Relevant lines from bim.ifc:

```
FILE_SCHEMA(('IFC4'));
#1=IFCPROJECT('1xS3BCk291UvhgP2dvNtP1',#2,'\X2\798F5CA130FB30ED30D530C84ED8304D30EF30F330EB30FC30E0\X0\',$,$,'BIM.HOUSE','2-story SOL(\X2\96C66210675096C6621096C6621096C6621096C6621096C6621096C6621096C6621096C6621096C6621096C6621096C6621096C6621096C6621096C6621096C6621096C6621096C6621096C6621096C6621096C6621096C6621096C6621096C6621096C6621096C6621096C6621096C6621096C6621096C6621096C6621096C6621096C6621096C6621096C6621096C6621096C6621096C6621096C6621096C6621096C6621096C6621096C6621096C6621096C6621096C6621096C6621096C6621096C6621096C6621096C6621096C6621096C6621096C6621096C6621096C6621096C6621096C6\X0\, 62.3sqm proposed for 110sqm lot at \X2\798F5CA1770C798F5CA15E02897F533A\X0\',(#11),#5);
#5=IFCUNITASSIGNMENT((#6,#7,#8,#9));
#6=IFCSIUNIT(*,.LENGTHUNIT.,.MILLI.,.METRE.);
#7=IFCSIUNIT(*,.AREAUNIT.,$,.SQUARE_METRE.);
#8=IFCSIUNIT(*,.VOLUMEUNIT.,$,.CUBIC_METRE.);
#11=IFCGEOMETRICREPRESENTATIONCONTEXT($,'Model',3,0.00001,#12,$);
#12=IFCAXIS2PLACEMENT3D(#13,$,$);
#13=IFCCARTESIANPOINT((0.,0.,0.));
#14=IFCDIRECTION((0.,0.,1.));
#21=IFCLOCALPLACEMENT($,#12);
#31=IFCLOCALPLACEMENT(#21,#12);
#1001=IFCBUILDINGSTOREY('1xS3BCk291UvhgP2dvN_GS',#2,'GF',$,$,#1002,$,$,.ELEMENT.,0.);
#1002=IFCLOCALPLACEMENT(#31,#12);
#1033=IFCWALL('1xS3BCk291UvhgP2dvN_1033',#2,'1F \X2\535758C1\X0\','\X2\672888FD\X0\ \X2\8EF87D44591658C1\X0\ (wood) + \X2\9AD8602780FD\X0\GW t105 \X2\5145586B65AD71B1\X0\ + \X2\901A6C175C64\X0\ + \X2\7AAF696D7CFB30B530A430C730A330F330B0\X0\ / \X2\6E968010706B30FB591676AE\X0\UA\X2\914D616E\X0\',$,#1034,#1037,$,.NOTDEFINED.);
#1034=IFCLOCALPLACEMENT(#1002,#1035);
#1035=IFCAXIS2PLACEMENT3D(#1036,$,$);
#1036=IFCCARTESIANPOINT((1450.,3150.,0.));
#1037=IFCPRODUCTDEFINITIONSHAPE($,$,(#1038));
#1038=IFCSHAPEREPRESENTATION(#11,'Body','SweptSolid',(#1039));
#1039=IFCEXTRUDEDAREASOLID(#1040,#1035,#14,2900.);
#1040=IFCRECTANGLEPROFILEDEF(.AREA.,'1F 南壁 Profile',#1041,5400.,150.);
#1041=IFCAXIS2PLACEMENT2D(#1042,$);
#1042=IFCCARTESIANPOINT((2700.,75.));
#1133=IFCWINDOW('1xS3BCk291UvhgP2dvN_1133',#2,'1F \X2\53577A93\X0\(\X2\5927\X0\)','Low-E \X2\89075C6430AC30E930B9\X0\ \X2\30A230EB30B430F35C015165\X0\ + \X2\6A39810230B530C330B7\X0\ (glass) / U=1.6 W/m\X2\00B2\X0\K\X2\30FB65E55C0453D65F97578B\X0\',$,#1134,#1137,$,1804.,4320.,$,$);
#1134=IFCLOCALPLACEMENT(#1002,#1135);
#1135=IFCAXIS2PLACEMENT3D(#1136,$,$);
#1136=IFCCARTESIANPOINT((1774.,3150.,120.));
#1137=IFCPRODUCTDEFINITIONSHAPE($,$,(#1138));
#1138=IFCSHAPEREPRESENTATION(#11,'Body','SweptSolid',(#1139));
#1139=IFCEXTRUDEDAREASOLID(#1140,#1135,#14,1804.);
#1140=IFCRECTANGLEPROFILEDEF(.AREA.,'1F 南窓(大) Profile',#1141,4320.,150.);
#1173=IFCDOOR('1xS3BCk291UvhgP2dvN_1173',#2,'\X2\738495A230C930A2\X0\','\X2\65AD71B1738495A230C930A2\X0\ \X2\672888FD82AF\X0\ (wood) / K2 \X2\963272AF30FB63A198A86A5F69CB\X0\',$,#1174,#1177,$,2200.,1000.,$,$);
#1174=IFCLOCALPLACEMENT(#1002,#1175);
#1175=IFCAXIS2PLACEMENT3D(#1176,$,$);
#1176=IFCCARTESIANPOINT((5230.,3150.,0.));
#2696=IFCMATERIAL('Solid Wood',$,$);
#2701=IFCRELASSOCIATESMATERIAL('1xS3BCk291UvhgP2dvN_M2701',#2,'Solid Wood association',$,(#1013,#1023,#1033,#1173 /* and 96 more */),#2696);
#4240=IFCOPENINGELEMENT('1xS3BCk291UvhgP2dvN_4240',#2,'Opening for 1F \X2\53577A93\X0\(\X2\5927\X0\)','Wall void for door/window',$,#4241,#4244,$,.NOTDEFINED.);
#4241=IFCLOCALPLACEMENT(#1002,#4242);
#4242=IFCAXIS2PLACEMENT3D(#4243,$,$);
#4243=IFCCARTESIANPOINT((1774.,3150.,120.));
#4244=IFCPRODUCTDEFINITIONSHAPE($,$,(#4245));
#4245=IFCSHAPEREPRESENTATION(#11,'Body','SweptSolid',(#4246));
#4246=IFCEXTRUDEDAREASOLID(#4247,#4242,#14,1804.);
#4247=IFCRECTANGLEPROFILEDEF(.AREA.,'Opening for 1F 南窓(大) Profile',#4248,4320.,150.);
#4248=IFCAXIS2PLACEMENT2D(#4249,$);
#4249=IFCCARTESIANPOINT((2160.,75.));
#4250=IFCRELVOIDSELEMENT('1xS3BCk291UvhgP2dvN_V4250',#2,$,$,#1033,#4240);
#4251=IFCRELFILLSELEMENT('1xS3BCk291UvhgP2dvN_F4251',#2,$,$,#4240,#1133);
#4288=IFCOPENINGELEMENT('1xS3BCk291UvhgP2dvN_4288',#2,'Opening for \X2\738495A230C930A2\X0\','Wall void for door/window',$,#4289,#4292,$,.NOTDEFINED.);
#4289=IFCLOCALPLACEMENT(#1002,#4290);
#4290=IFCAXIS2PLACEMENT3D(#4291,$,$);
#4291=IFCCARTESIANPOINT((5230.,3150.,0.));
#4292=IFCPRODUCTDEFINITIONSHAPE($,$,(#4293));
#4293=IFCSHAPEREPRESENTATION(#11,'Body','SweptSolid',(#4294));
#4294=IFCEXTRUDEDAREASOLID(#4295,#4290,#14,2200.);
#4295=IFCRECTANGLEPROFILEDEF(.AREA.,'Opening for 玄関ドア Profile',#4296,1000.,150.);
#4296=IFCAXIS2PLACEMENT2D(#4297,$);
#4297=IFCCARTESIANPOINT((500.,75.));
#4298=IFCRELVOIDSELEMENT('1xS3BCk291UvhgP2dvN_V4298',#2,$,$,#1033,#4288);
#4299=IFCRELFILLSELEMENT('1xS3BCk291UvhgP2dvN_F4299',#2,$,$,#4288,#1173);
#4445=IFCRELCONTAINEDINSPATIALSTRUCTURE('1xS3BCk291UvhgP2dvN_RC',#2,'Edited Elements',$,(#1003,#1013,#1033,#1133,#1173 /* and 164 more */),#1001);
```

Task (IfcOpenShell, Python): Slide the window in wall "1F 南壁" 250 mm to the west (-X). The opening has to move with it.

```python
import ifcopenshell
import ifcopenshell.api.geometry
import ifcopenshell.util.placement
import ifcopenshell.util.unit

model = ifcopenshell.open("bim.ifc")
unit_scale = ifcopenshell.util.unit.calculate_unit_scale(model)

window = model.by_guid("1xS3BCk291UvhgP2dvN_1133")
opening = window.FillsVoids[0].RelatingOpeningElement
wall = opening.VoidsElements[0].RelatingBuildingElement

wall_matrix = ifcopenshell.util.placement.get_local_placement(wall.ObjectPlacement)
shift = wall_matrix[:3, 0] * -0.25 / unit_scale
before = ifcopenshell.util.placement.get_local_placement(window.ObjectPlacement)[:3, 3].copy()

# The window is not placed relative to its opening, so move both.
for product in (opening, window):
    matrix = ifcopenshell.util.placement.get_local_placement(product.ObjectPlacement)
    matrix[:3, 3] += shift
    ifcopenshell.api.geometry.edit_object_placement(model, product=product, matrix=matrix, is_si=False)

after = ifcopenshell.util.placement.get_local_placement(window.ObjectPlacement)[:3, 3]
print("window moved by", (after - before).round(3) + 0.0)

model.write("bim_updated.ifc")
```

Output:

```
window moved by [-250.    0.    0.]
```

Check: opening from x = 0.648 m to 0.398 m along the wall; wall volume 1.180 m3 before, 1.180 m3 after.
